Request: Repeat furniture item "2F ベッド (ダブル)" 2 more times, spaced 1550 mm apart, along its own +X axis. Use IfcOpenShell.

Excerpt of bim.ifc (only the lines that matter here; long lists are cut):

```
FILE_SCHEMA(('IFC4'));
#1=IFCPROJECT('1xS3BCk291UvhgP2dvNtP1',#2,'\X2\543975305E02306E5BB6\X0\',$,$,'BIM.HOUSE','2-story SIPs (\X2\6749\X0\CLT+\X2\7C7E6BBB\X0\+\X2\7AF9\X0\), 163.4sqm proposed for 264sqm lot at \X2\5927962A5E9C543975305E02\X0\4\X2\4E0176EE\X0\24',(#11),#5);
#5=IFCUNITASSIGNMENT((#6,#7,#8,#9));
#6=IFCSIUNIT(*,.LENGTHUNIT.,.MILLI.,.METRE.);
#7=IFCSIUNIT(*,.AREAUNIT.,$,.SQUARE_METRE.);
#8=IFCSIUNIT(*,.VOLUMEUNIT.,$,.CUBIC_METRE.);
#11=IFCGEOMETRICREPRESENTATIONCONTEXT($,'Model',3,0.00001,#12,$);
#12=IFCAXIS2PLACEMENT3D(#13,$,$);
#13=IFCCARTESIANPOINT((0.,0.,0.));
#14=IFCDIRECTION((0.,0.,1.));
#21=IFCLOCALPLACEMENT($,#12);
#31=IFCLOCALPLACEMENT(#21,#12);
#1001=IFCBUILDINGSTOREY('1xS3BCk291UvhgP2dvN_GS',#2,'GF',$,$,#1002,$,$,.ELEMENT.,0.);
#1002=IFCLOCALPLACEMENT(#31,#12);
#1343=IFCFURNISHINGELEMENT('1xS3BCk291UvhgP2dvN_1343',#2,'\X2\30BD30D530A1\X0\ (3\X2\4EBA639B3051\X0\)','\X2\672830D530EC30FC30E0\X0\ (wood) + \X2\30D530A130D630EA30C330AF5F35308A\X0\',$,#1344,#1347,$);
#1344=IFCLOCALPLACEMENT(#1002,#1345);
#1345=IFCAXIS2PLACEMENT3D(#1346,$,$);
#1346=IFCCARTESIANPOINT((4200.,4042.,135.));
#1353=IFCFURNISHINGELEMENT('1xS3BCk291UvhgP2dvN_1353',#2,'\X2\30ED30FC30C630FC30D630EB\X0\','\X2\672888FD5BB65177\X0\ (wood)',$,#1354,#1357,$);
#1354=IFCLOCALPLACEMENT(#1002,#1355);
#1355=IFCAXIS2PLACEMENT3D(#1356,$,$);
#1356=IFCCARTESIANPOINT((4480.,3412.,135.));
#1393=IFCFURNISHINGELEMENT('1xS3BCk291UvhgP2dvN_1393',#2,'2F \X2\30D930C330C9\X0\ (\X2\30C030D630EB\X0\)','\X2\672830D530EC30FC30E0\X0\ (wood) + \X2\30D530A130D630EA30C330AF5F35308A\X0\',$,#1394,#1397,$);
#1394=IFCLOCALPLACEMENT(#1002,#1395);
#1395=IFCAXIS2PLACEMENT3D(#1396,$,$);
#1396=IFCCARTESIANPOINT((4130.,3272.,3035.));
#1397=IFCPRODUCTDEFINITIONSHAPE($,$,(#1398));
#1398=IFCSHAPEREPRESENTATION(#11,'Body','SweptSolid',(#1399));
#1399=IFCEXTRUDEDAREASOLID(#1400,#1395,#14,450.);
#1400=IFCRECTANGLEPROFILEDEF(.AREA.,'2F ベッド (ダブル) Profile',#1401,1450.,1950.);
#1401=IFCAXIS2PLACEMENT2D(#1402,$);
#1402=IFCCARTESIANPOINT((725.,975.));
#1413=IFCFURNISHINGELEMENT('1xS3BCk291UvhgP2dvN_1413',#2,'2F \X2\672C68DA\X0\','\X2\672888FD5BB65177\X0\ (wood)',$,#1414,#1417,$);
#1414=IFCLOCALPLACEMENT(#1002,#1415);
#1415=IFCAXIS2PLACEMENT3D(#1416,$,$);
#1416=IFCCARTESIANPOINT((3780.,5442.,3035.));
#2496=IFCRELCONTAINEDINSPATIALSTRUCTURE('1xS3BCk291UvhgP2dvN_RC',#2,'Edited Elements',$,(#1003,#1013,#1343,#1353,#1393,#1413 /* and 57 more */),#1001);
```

```python
import ifcopenshell
import ifcopenshell.api.geometry
import ifcopenshell.api.root
import ifcopenshell.util.element
import ifcopenshell.util.placement
import ifcopenshell.util.unit

model = ifcopenshell.open("bim.ifc")
unit_scale = ifcopenshell.util.unit.calculate_unit_scale(model)


def reuse_history(source, copy):
    """copy_class also copies each property set's owner history, people and application; keep the originals."""
    for rel in copy.IsDefinedBy:
        if rel.is_a("IfcRelDefinesByProperties") and (history := rel.RelatingPropertyDefinition.OwnerHistory):
            rel.RelatingPropertyDefinition.OwnerHistory = source.OwnerHistory
            ifcopenshell.util.element.remove_deep2(model, history)


source = model.by_guid("1xS3BCk291UvhgP2dvN_1393")
base = ifcopenshell.util.placement.get_local_placement(source.ObjectPlacement)
step = base[:3, 0] * 1.55 / unit_scale

for i in range(1, 3):
    copy = ifcopenshell.api.root.copy_class(model, product=source)
    copy.Representation = ifcopenshell.util.element.copy_deep(
        model, source.Representation, exclude=["IfcGeometricRepresentationContext", "IfcRepresentationMap"]
    )
    reuse_history(source, copy)
    matrix = base.copy()
    matrix[:3, 3] += i * step
    print("added at", matrix[:3, 3].round(3) + 0.0)
    ifcopenshell.api.geometry.edit_object_placement(model, product=copy, matrix=matrix, is_si=False)

model.write("bim_updated.ifc")
```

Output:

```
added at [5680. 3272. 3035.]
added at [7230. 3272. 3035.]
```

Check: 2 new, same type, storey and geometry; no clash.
